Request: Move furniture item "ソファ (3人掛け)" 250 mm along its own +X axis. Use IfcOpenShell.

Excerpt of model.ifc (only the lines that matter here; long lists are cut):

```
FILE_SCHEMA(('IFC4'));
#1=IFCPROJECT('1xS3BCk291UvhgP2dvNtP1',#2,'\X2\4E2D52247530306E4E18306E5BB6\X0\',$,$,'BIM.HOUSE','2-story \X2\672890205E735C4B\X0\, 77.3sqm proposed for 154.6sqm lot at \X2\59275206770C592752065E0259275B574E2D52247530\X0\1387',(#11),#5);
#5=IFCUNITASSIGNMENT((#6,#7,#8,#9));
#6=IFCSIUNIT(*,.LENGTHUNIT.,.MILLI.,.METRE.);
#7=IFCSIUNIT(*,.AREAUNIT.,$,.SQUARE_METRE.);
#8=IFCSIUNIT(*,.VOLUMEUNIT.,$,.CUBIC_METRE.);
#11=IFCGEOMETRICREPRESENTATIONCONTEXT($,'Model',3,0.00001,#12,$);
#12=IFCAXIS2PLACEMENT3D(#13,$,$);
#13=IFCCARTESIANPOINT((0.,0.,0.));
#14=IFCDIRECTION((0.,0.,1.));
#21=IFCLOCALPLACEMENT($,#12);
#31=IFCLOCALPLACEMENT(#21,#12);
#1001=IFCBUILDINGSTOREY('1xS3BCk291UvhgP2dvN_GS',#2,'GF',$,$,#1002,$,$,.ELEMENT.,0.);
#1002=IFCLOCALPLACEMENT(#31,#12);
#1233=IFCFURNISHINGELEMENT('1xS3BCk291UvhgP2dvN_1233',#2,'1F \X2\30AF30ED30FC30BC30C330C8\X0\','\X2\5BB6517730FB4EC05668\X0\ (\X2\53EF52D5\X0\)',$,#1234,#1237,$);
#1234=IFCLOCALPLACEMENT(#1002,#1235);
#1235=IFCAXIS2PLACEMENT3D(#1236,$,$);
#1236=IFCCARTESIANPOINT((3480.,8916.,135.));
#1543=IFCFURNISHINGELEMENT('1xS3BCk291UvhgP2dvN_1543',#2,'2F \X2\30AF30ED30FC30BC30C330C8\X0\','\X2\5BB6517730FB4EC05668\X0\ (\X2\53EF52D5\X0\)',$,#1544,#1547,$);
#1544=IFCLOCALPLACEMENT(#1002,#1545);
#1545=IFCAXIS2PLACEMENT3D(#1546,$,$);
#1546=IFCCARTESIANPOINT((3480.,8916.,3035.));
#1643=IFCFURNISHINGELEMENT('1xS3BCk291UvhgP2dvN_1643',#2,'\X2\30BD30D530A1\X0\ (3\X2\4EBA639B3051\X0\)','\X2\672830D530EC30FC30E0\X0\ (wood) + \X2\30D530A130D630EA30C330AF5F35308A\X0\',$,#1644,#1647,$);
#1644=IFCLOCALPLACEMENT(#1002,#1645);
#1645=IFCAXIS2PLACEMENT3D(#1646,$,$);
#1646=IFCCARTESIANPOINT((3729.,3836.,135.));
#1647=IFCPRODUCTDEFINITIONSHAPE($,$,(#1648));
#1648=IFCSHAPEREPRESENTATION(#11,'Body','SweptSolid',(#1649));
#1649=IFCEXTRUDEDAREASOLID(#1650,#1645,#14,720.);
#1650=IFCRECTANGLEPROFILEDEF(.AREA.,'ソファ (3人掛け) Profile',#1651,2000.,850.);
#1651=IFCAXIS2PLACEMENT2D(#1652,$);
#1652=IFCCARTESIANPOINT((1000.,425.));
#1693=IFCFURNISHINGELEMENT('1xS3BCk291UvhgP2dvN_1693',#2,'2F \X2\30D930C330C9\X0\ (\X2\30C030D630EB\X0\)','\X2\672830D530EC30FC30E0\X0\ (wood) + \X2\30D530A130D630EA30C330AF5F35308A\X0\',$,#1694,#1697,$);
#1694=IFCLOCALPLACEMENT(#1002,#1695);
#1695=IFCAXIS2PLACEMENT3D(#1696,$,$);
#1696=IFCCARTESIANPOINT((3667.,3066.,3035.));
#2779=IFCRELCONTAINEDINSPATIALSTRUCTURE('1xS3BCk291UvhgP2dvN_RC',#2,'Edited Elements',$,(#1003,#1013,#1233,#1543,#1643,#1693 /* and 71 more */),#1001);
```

```python
import ifcopenshell
import ifcopenshell.api.geometry
import ifcopenshell.util.placement
import ifcopenshell.util.unit

model = ifcopenshell.open("model.ifc")
unit_scale = ifcopenshell.util.unit.calculate_unit_scale(model)

item = model.by_guid("1xS3BCk291UvhgP2dvN_1643")
matrix = ifcopenshell.util.placement.get_local_placement(item.ObjectPlacement)
matrix[:3, 3] += matrix[:3, 0] * 0.25 / unit_scale
ifcopenshell.api.geometry.edit_object_placement(model, product=item, matrix=matrix, is_si=False)

print(ifcopenshell.util.placement.get_local_placement(item.ObjectPlacement).round(3) + 0.0)

model.write("model_edited.ifc")
```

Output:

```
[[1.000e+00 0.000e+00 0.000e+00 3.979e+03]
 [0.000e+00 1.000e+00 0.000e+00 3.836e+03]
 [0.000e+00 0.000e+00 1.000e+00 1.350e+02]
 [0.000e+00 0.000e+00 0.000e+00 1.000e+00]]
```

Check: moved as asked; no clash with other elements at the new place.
